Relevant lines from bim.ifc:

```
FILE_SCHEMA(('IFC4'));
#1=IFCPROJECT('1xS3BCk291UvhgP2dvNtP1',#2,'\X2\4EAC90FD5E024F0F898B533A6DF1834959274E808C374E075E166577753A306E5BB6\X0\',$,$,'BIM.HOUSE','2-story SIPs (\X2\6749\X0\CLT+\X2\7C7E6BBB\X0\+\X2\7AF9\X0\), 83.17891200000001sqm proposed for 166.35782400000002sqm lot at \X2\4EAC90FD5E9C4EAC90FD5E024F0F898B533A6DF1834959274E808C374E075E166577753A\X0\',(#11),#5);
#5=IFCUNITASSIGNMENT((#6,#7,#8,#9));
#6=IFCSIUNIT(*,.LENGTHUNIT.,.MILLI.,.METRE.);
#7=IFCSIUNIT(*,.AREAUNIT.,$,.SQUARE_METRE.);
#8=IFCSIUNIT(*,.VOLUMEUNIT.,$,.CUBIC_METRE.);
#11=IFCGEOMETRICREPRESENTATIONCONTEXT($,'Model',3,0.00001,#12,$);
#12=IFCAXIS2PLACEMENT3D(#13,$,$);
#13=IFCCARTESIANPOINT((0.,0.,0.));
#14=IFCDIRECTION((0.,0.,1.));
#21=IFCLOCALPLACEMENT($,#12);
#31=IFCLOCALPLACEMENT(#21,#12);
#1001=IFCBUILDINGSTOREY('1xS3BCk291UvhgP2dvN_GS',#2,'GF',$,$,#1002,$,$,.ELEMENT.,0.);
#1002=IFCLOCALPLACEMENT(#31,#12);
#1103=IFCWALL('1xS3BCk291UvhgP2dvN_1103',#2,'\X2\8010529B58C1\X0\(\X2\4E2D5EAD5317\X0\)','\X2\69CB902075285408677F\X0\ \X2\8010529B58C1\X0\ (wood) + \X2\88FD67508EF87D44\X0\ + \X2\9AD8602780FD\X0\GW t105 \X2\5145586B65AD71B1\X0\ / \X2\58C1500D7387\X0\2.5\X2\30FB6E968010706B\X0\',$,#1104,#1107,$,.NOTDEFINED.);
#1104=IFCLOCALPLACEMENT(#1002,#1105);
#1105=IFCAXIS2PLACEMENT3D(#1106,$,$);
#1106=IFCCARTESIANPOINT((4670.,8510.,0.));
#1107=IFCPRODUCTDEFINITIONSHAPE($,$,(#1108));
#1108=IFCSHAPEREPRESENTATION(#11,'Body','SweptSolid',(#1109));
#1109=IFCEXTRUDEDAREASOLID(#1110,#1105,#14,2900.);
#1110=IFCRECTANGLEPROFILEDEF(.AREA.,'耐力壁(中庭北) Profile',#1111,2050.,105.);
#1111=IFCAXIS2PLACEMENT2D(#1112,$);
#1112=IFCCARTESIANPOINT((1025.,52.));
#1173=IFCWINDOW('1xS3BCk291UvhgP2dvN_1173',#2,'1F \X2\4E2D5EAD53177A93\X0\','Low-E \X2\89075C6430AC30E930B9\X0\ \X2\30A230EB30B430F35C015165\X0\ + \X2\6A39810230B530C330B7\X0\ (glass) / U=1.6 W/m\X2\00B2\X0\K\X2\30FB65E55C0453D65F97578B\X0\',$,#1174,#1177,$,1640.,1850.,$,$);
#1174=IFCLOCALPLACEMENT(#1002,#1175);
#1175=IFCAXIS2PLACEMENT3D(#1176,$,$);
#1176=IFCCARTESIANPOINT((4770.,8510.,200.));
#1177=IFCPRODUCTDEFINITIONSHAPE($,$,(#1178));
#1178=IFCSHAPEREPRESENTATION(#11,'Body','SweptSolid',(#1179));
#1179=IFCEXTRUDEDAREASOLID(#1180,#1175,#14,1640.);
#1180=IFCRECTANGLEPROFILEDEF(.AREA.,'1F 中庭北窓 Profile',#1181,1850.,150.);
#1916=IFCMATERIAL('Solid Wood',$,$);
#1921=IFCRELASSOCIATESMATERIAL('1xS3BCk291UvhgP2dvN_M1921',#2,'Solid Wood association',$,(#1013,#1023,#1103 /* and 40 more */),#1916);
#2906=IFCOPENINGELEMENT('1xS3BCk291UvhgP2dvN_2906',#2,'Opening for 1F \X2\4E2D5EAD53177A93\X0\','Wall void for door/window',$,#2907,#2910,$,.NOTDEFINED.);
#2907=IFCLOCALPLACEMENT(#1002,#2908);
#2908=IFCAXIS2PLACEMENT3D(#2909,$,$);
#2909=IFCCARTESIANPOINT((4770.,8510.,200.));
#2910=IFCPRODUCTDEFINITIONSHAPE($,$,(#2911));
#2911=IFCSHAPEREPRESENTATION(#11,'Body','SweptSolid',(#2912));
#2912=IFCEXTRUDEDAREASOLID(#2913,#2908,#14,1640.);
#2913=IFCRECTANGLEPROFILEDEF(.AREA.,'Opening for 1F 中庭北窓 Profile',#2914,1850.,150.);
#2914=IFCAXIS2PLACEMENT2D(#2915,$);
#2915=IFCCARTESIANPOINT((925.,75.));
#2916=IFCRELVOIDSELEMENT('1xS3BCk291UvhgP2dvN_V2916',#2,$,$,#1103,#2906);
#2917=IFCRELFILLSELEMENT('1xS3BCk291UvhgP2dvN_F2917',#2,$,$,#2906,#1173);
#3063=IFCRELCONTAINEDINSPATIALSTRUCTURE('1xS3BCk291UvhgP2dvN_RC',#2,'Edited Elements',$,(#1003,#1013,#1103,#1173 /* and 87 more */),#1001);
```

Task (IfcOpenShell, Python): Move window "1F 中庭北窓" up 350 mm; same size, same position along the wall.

```python
import numpy as np
import ifcopenshell
import ifcopenshell.api.geometry
import ifcopenshell.util.placement
import ifcopenshell.util.unit

model = ifcopenshell.open("bim.ifc")
unit_scale = ifcopenshell.util.unit.calculate_unit_scale(model)

window = model.by_guid("1xS3BCk291UvhgP2dvN_1173")
opening = window.FillsVoids[0].RelatingOpeningElement
dz = 350.0

shift = np.array([0.0, 0.0, dz])
# The window is not placed relative to its opening, so move both.
for product in (opening, window):
    matrix = ifcopenshell.util.placement.get_local_placement(product.ObjectPlacement)
    matrix[:3, 3] += shift
    ifcopenshell.api.geometry.edit_object_placement(model, product=product, matrix=matrix, is_si=False)

print(f"moved by {dz * unit_scale:+.3f} m")

model.write("bim_rev.ifc")
```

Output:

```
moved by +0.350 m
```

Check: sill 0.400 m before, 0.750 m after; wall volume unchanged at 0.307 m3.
